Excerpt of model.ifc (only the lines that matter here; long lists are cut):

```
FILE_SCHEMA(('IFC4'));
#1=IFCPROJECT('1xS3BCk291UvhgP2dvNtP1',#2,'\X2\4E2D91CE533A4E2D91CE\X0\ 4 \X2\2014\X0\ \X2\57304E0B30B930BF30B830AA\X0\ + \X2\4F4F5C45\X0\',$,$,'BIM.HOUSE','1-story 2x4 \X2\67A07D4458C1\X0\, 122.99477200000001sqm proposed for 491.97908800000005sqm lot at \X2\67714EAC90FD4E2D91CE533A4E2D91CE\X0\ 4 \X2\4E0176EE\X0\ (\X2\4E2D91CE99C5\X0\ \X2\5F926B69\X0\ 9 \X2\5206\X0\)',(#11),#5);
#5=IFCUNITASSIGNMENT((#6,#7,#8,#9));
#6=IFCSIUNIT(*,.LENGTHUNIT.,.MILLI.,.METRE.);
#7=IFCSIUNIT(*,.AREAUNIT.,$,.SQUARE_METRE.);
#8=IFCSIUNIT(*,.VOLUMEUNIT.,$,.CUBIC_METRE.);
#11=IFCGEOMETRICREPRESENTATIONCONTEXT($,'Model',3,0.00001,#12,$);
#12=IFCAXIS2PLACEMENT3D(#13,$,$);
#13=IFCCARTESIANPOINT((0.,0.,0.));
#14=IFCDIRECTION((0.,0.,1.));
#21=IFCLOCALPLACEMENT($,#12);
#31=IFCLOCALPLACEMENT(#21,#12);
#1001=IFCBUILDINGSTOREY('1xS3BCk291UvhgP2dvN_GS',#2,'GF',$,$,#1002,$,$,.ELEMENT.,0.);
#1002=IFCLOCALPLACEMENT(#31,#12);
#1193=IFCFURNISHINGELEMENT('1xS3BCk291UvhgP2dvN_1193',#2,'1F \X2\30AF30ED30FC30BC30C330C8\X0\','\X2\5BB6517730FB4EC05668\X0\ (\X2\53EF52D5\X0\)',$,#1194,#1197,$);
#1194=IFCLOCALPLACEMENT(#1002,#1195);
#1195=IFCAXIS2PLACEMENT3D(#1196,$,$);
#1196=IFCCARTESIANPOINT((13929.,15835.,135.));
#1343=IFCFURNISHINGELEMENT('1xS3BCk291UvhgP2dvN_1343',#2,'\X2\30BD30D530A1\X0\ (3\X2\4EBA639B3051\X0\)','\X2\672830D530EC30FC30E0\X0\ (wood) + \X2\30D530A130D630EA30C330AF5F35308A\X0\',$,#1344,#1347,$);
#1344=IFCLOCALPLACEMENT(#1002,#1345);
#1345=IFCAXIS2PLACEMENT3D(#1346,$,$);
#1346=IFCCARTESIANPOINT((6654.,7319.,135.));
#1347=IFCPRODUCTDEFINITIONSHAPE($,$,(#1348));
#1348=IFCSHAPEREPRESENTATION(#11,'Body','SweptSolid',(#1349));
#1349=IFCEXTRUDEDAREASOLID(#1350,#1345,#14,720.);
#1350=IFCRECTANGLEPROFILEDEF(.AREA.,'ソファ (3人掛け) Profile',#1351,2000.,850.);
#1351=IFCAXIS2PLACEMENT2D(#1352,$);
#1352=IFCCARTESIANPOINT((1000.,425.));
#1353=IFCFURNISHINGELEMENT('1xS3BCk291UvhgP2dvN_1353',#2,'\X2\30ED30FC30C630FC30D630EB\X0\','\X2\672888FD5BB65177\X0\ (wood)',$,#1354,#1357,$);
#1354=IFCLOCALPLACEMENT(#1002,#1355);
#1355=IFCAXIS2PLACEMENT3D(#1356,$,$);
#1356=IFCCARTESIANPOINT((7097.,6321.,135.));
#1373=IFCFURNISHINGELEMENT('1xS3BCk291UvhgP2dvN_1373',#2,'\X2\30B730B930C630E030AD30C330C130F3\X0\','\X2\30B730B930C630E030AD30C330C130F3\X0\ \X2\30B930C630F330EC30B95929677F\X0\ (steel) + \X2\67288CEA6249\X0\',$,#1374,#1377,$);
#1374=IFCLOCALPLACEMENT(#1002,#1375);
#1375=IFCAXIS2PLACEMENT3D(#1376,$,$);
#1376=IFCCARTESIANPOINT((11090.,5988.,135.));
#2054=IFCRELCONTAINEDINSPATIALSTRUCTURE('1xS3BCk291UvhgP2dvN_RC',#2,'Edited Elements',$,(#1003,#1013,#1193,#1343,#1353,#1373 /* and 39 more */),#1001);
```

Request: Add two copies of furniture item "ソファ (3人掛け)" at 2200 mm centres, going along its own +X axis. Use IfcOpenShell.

```python
import ifcopenshell
import ifcopenshell.api.geometry
import ifcopenshell.api.root
import ifcopenshell.util.element
import ifcopenshell.util.placement
import ifcopenshell.util.unit

model = ifcopenshell.open("model.ifc")
unit_scale = ifcopenshell.util.unit.calculate_unit_scale(model)


def reuse_history(source, copy):
    """copy_class also copies each property set's owner history, people and application; keep the originals."""
    for rel in copy.IsDefinedBy:
        if rel.is_a("IfcRelDefinesByProperties") and (history := rel.RelatingPropertyDefinition.OwnerHistory):
            rel.RelatingPropertyDefinition.OwnerHistory = source.OwnerHistory
            ifcopenshell.util.element.remove_deep2(model, history)


source = model.by_guid("1xS3BCk291UvhgP2dvN_1343")
base = ifcopenshell.util.placement.get_local_placement(source.ObjectPlacement)
step = base[:3, 0] * 2.2 / unit_scale

for i in range(1, 3):
    copy = ifcopenshell.api.root.copy_class(model, product=source)
    copy.Representation = ifcopenshell.util.element.copy_deep(
        model, source.Representation, exclude=["IfcGeometricRepresentationContext", "IfcRepresentationMap"]
    )
    reuse_history(source, copy)
    matrix = base.copy()
    matrix[:3, 3] += i * step
    print("added at", matrix[:3, 3].round(3) + 0.0)
    ifcopenshell.api.geometry.edit_object_placement(model, product=copy, matrix=matrix, is_si=False)

model.write("model_v2.ifc")
```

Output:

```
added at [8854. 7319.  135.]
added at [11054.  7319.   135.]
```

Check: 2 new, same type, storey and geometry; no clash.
